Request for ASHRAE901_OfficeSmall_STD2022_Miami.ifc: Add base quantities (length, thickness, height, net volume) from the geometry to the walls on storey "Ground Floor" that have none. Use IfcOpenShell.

First a look at what the model holds.

```python
import ifcopenshell
import ifcopenshell.util.element
import ifcopenshell.util.unit

model = ifcopenshell.open("ASHRAE901_OfficeSmall_STD2022_Miami.ifc")
print(model.schema)
for unit_type in ("LENGTHUNIT", "AREAUNIT", "VOLUMEUNIT"):
    print(unit_type, ifcopenshell.util.unit.calculate_unit_scale(model, unit_type))
storey = next(s for s in model.by_type("IfcBuildingStorey") if s.Name == "Ground Floor")
walls = [e for e in ifcopenshell.util.element.get_decomposition(storey) if e.is_a("IfcWall")]
for e in sorted(walls, key=lambda e: e.id()):
    print(e.id(), e.is_a(), e.Name, list(ifcopenshell.util.element.get_psets(e, qtos_only=True)), sep=" | ")
```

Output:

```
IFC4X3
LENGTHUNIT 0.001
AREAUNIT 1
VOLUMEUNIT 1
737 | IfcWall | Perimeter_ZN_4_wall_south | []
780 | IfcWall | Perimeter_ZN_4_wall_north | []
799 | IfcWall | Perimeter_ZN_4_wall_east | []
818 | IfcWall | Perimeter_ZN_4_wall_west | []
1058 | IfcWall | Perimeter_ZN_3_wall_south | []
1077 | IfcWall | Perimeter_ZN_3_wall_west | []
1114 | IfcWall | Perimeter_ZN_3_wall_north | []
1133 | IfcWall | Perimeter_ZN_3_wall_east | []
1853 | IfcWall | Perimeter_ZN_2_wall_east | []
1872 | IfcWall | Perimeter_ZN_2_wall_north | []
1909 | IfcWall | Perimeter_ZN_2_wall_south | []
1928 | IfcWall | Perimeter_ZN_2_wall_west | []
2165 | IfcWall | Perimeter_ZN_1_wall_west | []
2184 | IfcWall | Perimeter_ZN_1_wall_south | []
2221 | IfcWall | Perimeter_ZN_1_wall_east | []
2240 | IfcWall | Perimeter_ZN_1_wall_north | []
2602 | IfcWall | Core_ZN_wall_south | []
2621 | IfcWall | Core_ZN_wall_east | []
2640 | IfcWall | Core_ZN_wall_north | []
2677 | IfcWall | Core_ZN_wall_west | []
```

```python
import ifcopenshell
import ifcopenshell.api.pset
import ifcopenshell.geom
import ifcopenshell.util.element
import ifcopenshell.util.shape
import ifcopenshell.util.unit

model = ifcopenshell.open("ASHRAE901_OfficeSmall_STD2022_Miami.ifc")
unit_scale = ifcopenshell.util.unit.calculate_unit_scale(model)
volume_scale = ifcopenshell.util.unit.calculate_unit_scale(model, "VOLUMEUNIT")
settings = ifcopenshell.geom.settings()

storey = next(s for s in model.by_type("IfcBuildingStorey") if s.Name == "Ground Floor")
walls = [e for e in ifcopenshell.util.element.get_decomposition(storey) if e.is_a("IfcWall")]

for e in sorted(walls, key=lambda e: e.id()):
    if ifcopenshell.util.element.get_psets(e, qtos_only=True, should_inherit=False):
        continue
    # Geometry comes back in metres, in the element's own axes.
    shape = ifcopenshell.geom.create_shape(settings, e)
    values = {
        "Length": ifcopenshell.util.shape.get_x(shape.geometry) / unit_scale,
        "Width": ifcopenshell.util.shape.get_y(shape.geometry) / unit_scale,
        "Height": ifcopenshell.util.shape.get_z(shape.geometry) / unit_scale,
        "NetVolume": ifcopenshell.util.shape.get_volume(shape.geometry) / volume_scale,
    }
    qto = ifcopenshell.api.pset.add_qto(model, product=e, name="Qto_WallBaseQuantities")
    ifcopenshell.api.pset.edit_qto(model, qto=qto, properties=values)
    print(e.id(), {k: round(v, 3) for k, v in values.items()})

model.write("ASHRAE901_OfficeSmall_STD2022_Miami_rev.ifc")
```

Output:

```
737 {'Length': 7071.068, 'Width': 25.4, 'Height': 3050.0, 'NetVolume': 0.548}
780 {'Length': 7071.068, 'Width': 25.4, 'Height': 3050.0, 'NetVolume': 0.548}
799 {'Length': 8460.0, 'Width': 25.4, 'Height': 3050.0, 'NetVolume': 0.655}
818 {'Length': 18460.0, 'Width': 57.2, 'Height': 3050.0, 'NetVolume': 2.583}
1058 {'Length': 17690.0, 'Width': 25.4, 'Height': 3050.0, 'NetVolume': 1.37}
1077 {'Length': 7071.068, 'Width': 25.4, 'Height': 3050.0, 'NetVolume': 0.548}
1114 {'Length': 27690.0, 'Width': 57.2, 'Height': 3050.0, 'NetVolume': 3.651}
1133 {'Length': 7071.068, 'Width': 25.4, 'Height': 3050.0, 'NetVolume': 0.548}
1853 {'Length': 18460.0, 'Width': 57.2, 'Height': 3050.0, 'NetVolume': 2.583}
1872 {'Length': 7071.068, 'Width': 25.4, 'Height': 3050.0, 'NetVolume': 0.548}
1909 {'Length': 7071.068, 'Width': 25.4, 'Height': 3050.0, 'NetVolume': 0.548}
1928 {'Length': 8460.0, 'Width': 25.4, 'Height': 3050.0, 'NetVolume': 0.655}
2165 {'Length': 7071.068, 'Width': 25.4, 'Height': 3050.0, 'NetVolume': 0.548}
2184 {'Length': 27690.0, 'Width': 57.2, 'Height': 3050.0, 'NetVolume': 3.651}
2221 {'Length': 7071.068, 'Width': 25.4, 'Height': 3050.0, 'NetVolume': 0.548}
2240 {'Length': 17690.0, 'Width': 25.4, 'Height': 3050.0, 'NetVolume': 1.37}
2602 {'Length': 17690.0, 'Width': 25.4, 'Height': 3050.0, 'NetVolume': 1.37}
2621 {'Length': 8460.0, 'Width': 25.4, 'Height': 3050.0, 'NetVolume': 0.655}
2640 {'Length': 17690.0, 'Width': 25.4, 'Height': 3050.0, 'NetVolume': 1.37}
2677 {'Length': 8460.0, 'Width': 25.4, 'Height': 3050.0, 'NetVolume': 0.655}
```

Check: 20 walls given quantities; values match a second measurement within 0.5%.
